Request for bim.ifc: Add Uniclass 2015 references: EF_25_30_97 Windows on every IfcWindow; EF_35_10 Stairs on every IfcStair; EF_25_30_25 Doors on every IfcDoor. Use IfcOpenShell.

First a look at what the model holds.

```python
import ifcopenshell

model = ifcopenshell.open("bim.ifc")
print(model.schema)
print("classifications:", [c.Name for c in model.by_type("IfcClassification")])
for ifc_class in ("IfcDoor", "IfcRoof", "IfcStair", "IfcWall", "IfcWindow"):
    print(ifc_class, len(model.by_type(ifc_class)))
```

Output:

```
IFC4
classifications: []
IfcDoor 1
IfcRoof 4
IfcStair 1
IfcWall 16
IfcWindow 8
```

```python
import ifcopenshell
import ifcopenshell.api.classification

model = ifcopenshell.open("bim.ifc")

system = ifcopenshell.api.classification.add_classification(model, classification="Uniclass 2015")

codes = {
    "IfcWindow": ("EF_25_30_97", "Windows"),
    "IfcStair": ("EF_35_10", "Stairs"),
    "IfcDoor": ("EF_25_30_25", "Doors"),
}
for ifc_class, (code, name) in codes.items():
    products = model.by_type(ifc_class)
    ifcopenshell.api.classification.add_reference(
        model, products=products, classification=system, identification=code, name=name
    )
    print(code, len(products))

model.write("bim_edited.ifc")
```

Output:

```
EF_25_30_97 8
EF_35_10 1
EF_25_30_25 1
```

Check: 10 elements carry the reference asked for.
